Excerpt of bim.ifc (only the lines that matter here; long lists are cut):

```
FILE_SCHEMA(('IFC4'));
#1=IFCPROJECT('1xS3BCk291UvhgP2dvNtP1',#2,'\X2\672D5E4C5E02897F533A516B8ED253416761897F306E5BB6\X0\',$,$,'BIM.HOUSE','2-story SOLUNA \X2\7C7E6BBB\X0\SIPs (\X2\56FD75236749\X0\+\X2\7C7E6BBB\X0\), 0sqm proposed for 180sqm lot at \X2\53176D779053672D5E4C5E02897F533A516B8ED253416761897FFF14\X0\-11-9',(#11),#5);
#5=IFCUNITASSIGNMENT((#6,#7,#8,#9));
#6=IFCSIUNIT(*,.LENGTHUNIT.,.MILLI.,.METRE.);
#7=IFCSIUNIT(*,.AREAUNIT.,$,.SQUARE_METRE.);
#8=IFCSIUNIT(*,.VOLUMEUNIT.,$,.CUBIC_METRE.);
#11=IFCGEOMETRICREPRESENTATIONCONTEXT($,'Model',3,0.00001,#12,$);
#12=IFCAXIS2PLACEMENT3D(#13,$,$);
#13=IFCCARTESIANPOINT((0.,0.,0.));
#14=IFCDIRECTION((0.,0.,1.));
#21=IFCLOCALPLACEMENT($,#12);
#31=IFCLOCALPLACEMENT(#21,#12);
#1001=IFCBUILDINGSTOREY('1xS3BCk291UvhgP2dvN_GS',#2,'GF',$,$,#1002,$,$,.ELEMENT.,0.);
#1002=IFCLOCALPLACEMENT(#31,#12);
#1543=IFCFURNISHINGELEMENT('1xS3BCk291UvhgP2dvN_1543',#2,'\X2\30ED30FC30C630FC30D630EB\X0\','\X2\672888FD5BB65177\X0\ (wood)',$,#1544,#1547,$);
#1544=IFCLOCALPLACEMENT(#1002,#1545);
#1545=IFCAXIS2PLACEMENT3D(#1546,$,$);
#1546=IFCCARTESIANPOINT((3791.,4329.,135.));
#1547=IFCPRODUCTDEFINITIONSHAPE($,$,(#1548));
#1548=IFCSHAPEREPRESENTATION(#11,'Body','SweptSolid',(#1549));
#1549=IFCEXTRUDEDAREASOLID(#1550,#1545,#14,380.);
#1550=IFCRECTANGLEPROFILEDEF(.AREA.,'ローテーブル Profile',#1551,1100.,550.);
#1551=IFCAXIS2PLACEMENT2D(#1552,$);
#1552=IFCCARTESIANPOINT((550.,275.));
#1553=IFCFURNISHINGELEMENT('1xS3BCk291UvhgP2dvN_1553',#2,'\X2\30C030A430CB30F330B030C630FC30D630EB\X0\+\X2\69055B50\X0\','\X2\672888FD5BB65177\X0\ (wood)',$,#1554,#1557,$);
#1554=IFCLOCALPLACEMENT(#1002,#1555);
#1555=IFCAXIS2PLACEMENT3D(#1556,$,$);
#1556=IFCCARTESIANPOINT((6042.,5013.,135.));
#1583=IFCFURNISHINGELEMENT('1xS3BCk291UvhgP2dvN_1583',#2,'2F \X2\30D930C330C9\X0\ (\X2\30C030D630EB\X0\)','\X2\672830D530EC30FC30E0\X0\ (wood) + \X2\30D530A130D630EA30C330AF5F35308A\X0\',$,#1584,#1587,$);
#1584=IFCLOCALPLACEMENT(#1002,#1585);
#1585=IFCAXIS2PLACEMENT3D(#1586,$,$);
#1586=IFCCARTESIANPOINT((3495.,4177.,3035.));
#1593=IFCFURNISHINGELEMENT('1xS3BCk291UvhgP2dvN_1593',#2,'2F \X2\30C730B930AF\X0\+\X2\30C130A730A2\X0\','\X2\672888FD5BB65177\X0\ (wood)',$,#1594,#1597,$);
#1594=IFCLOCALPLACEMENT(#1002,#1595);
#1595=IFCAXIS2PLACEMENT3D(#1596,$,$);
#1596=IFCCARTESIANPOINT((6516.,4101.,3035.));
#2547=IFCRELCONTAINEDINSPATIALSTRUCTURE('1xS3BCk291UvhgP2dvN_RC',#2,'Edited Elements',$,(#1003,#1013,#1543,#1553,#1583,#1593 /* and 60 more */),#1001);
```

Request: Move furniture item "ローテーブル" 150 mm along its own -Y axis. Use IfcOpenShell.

```python
import ifcopenshell
import ifcopenshell.api.geometry
import ifcopenshell.util.placement
import ifcopenshell.util.unit

model = ifcopenshell.open("bim.ifc")
unit_scale = ifcopenshell.util.unit.calculate_unit_scale(model)

item = model.by_guid("1xS3BCk291UvhgP2dvN_1543")
matrix = ifcopenshell.util.placement.get_local_placement(item.ObjectPlacement)
matrix[:3, 3] -= matrix[:3, 1] * 0.15 / unit_scale
ifcopenshell.api.geometry.edit_object_placement(model, product=item, matrix=matrix, is_si=False)

print(ifcopenshell.util.placement.get_local_placement(item.ObjectPlacement).round(3) + 0.0)

model.write("bim_rev.ifc")
```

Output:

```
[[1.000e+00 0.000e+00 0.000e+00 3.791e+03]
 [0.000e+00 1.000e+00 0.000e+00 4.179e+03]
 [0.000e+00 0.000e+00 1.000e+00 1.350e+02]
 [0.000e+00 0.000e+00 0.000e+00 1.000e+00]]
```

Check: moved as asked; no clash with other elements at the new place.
